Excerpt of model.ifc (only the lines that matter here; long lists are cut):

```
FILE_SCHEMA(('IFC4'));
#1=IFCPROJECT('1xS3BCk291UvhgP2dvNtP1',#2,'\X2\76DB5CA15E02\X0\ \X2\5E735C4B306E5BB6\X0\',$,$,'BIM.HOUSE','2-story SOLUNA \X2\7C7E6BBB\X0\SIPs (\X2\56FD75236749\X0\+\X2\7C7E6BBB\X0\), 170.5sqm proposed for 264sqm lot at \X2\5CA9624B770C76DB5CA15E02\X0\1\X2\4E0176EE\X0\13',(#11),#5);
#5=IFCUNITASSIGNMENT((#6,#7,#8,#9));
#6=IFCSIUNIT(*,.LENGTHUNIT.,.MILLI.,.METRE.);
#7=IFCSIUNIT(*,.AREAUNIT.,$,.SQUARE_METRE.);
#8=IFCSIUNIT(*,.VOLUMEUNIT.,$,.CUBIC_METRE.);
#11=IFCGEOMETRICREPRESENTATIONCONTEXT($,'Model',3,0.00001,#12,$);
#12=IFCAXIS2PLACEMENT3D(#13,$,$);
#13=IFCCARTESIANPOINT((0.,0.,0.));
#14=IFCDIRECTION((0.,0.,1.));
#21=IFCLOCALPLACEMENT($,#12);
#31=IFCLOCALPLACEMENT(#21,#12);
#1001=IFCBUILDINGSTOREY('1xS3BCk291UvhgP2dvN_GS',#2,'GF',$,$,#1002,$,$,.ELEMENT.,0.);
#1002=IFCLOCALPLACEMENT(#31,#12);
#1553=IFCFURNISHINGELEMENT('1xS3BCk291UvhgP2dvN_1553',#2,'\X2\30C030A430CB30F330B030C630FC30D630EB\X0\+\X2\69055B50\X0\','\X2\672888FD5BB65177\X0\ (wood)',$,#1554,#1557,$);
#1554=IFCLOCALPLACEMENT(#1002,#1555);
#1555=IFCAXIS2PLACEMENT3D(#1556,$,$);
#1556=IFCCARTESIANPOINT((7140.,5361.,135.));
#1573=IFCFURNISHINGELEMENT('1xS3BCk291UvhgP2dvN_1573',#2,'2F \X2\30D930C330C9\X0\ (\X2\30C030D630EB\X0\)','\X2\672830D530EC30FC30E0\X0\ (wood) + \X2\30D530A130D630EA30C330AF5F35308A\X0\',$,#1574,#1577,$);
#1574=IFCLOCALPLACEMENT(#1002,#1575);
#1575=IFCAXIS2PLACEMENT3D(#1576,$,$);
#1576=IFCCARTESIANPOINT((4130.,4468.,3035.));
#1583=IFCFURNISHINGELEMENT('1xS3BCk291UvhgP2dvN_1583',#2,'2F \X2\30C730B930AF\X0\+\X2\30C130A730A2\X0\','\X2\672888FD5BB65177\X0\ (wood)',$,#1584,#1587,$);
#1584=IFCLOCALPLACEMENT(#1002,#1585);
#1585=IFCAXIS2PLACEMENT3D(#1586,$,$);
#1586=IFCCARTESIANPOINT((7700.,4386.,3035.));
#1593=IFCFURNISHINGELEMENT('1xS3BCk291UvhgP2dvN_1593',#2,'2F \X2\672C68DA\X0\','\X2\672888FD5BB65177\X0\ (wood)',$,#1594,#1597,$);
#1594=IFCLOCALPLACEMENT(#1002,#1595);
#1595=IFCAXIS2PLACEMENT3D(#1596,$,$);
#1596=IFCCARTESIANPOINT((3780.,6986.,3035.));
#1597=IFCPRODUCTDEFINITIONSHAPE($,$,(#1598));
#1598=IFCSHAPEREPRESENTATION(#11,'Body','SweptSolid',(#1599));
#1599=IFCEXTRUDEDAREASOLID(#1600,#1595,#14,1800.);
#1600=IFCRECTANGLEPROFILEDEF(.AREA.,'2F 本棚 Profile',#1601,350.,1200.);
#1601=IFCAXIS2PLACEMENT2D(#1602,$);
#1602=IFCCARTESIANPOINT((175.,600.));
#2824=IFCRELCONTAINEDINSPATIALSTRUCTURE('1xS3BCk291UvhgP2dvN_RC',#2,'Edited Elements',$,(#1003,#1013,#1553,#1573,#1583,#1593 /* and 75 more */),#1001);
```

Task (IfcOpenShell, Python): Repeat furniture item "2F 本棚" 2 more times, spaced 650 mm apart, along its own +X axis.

```python
import ifcopenshell
import ifcopenshell.api.geometry
import ifcopenshell.api.root
import ifcopenshell.util.element
import ifcopenshell.util.placement

model = ifcopenshell.open("model.ifc")


def reuse_history(source, copy):
    """copy_class also copies each property set's owner history, people and application; keep the originals."""
    for rel in copy.IsDefinedBy:
        if rel.is_a("IfcRelDefinesByProperties") and (history := rel.RelatingPropertyDefinition.OwnerHistory):
            rel.RelatingPropertyDefinition.OwnerHistory = source.OwnerHistory
            ifcopenshell.util.element.remove_deep2(model, history)


source = model.by_guid("1xS3BCk291UvhgP2dvN_1593")
base = ifcopenshell.util.placement.get_local_placement(source.ObjectPlacement)
step = base[:3, 0] * 650.0

for i in range(1, 3):
    copy = ifcopenshell.api.root.copy_class(model, product=source)
    copy.Representation = ifcopenshell.util.element.copy_deep(
        model, source.Representation, exclude=["IfcGeometricRepresentationContext", "IfcRepresentationMap"]
    )
    reuse_history(source, copy)
    matrix = base.copy()
    matrix[:3, 3] += i * step
    print("added at", matrix[:3, 3].round(3) + 0.0)
    ifcopenshell.api.geometry.edit_object_placement(model, product=copy, matrix=matrix, is_si=False)

model.write("model_rev.ifc")
```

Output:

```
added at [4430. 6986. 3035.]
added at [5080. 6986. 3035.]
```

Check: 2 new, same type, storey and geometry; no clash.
